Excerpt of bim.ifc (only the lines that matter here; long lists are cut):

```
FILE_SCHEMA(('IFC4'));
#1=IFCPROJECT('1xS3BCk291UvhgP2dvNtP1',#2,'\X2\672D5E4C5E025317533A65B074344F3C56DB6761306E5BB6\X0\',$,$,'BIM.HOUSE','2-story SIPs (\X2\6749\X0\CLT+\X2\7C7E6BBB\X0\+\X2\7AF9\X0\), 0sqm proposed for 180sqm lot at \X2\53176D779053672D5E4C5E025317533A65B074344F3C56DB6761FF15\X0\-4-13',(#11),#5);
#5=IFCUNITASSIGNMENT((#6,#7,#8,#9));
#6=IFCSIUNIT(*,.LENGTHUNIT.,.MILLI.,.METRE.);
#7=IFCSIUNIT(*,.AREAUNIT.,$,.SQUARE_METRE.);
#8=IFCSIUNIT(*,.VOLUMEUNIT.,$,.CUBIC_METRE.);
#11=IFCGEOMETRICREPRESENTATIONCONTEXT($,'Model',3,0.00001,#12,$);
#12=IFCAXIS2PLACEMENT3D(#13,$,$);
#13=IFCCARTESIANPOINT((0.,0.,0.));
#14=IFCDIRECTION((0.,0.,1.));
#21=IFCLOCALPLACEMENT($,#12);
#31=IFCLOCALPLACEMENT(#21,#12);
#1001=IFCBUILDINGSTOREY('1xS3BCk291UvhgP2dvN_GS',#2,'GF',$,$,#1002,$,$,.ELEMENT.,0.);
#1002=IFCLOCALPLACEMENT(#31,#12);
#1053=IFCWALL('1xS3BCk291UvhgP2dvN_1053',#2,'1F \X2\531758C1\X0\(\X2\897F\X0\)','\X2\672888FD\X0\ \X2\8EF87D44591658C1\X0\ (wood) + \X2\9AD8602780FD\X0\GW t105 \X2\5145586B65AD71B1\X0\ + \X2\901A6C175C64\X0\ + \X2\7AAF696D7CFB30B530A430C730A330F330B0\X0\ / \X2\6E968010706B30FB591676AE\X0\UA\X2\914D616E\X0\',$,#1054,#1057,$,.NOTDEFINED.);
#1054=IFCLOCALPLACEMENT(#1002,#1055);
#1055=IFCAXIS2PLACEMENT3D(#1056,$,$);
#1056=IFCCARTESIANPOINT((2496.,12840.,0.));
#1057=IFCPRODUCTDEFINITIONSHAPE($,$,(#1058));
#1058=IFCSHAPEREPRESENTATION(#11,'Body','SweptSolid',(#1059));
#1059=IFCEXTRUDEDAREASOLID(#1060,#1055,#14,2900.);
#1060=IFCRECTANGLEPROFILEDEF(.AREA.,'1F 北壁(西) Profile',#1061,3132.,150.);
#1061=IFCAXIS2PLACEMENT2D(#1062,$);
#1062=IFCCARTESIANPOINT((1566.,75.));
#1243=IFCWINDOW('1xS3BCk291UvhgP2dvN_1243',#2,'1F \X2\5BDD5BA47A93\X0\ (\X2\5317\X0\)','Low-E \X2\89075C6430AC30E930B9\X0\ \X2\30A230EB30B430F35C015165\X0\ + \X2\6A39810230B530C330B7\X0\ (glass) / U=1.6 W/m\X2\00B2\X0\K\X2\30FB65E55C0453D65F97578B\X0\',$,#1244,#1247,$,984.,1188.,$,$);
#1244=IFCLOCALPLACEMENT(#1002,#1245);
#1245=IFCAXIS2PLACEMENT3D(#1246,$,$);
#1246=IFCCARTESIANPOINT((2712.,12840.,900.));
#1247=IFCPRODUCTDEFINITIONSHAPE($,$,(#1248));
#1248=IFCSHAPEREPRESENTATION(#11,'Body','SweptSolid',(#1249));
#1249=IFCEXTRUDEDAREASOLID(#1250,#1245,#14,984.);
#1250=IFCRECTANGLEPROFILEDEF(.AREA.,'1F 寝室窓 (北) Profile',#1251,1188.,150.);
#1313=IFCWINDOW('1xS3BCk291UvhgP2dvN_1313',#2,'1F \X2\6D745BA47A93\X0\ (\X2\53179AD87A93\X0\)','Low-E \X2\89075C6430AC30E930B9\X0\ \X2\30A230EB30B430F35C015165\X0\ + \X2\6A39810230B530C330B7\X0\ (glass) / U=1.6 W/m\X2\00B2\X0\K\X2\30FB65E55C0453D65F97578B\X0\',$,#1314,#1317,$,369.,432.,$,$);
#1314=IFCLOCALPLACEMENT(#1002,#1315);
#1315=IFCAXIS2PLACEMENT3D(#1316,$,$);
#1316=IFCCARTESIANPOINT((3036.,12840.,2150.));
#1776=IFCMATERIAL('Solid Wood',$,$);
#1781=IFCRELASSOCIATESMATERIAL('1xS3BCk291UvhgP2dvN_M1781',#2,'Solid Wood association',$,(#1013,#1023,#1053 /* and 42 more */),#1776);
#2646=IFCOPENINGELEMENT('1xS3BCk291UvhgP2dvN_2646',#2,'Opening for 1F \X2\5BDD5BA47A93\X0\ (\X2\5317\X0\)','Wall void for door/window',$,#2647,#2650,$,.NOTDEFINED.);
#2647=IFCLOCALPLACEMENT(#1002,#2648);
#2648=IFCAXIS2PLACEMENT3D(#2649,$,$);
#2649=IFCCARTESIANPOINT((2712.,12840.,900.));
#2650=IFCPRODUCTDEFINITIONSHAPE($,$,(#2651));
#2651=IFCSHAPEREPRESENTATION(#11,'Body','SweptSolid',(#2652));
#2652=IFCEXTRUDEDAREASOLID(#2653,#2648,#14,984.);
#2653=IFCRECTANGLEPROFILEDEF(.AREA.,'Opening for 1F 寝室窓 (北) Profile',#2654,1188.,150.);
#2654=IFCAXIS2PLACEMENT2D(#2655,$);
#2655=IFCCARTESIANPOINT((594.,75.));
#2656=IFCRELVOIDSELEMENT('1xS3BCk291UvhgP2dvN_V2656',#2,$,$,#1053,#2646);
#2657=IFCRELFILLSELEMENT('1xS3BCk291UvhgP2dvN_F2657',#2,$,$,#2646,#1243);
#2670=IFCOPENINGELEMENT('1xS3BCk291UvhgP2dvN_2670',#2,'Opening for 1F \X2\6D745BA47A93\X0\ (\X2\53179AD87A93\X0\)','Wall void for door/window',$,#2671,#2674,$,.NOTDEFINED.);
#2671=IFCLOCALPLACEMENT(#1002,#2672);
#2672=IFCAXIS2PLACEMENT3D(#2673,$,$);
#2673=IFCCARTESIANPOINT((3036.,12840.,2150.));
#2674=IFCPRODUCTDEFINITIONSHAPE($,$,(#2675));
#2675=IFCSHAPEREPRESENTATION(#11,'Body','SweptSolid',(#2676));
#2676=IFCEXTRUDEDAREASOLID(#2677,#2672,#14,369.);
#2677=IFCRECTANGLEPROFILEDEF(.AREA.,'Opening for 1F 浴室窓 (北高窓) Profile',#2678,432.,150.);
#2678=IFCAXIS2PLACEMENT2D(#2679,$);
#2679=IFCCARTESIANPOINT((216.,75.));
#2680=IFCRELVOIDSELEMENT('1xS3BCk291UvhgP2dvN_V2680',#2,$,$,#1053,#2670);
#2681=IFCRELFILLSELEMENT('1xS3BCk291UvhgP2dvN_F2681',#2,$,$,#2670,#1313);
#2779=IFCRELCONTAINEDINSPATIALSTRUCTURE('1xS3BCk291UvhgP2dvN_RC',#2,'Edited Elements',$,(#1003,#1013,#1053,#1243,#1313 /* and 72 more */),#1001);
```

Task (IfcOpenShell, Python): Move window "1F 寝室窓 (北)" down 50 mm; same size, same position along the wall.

```python
import numpy as np
import ifcopenshell
import ifcopenshell.api.geometry
import ifcopenshell.util.placement
import ifcopenshell.util.unit

model = ifcopenshell.open("bim.ifc")
unit_scale = ifcopenshell.util.unit.calculate_unit_scale(model)

window = model.by_guid("1xS3BCk291UvhgP2dvN_1243")
opening = window.FillsVoids[0].RelatingOpeningElement
dz = -50.0

shift = np.array([0.0, 0.0, dz])
# The window is not placed relative to its opening, so move both.
for product in (opening, window):
    matrix = ifcopenshell.util.placement.get_local_placement(product.ObjectPlacement)
    matrix[:3, 3] += shift
    ifcopenshell.api.geometry.edit_object_placement(model, product=product, matrix=matrix, is_si=False)

print(f"moved by {dz * unit_scale:+.3f} m")

model.write("bim_rev.ifc")
```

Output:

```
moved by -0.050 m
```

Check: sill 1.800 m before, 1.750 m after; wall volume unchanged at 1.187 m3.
